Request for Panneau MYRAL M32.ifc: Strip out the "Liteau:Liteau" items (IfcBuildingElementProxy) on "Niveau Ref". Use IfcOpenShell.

First a look at what the model holds.

```python
import ifcopenshell
import ifcopenshell.util.element

model = ifcopenshell.open("Panneau MYRAL M32.ifc")
print(model.schema)
storey = next(s for s in model.by_type("IfcBuildingStorey") if s.Name == "Niveau Ref")
proxies = [e for e in ifcopenshell.util.element.get_decomposition(storey) if e.is_a("IfcBuildingElementProxy")]
seen = {}
for e in proxies:
    element_type = ifcopenshell.util.element.get_type(e)
    name = element_type.Name if element_type not in (None, e) else None
    seen[name] = seen.get(name, 0) + 1
for name, count in sorted(seen.items(), key=str):
    print(count, "x", name)
```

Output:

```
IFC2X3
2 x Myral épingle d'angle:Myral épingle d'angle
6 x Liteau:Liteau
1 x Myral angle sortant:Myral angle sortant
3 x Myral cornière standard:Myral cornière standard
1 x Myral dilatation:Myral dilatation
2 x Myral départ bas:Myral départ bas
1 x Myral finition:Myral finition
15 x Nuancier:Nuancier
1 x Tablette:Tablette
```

```python
import ifcopenshell
import ifcopenshell.api.root
import ifcopenshell.util.element

model = ifcopenshell.open("Panneau MYRAL M32.ifc")

storey = next(s for s in model.by_type("IfcBuildingStorey") if s.Name == "Niveau Ref")
proxies = [e for e in ifcopenshell.util.element.get_decomposition(storey) if e.is_a("IfcBuildingElementProxy")]
targets = [e for e in proxies if (t := ifcopenshell.util.element.get_type(e)) not in (None, e) and t.Name == "Liteau:Liteau"]

for e in targets:
    ifcopenshell.api.root.remove_product(model, product=e)
print(len(targets), "removed")

model.write("Panneau MYRAL M32-out.ifc")
```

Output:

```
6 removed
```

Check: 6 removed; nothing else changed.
